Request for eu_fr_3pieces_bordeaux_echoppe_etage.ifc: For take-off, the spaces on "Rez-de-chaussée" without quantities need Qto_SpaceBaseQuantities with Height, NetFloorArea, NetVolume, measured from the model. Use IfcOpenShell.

First a look at what the model holds.

```python
import ifcopenshell
import ifcopenshell.util.element
import ifcopenshell.util.unit

model = ifcopenshell.open("eu_fr_3pieces_bordeaux_echoppe_etage.ifc")
print(model.schema)
for unit_type in ("LENGTHUNIT", "AREAUNIT", "VOLUMEUNIT"):
    print(unit_type, ifcopenshell.util.unit.calculate_unit_scale(model, unit_type))
storey = next(s for s in model.by_type("IfcBuildingStorey") if s.Name == "Rez-de-chaussée")
spaces = [e for e in ifcopenshell.util.element.get_decomposition(storey) if e.is_a("IfcSpace")]
for e in sorted(spaces, key=lambda e: e.id()):
    print(e.id(), e.is_a(), e.Name, list(ifcopenshell.util.element.get_psets(e, qtos_only=True)), sep=" | ")
```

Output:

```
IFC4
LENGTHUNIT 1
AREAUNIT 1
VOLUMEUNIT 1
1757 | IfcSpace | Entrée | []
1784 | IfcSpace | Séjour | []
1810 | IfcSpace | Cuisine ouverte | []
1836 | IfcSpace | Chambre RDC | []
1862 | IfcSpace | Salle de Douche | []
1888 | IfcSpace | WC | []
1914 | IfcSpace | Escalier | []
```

```python
import ifcopenshell
import ifcopenshell.api.pset
import ifcopenshell.geom
import ifcopenshell.util.element
import ifcopenshell.util.shape
import ifcopenshell.util.unit

model = ifcopenshell.open("eu_fr_3pieces_bordeaux_echoppe_etage.ifc")
unit_scale = ifcopenshell.util.unit.calculate_unit_scale(model)
area_scale = ifcopenshell.util.unit.calculate_unit_scale(model, "AREAUNIT")
volume_scale = ifcopenshell.util.unit.calculate_unit_scale(model, "VOLUMEUNIT")
settings = ifcopenshell.geom.settings()

storey = next(s for s in model.by_type("IfcBuildingStorey") if s.Name == "Rez-de-chaussée")
spaces = [e for e in ifcopenshell.util.element.get_decomposition(storey) if e.is_a("IfcSpace")]

for e in sorted(spaces, key=lambda e: e.id()):
    if ifcopenshell.util.element.get_psets(e, qtos_only=True, should_inherit=False):
        continue
    # Geometry comes back in metres, in the element's own axes.
    shape = ifcopenshell.geom.create_shape(settings, e)
    values = {
        "Height": ifcopenshell.util.shape.get_z(shape.geometry) / unit_scale,
        "NetFloorArea": ifcopenshell.util.shape.get_footprint_area(shape.geometry) / area_scale,
        "NetVolume": ifcopenshell.util.shape.get_volume(shape.geometry) / volume_scale,
    }
    qto = ifcopenshell.api.pset.add_qto(model, product=e, name="Qto_SpaceBaseQuantities")
    ifcopenshell.api.pset.edit_qto(model, qto=qto, properties=values)
    print(e.id(), {k: round(v, 3) for k, v in values.items()})

model.write("eu_fr_3pieces_bordeaux_echoppe_etage_v2.ifc")
```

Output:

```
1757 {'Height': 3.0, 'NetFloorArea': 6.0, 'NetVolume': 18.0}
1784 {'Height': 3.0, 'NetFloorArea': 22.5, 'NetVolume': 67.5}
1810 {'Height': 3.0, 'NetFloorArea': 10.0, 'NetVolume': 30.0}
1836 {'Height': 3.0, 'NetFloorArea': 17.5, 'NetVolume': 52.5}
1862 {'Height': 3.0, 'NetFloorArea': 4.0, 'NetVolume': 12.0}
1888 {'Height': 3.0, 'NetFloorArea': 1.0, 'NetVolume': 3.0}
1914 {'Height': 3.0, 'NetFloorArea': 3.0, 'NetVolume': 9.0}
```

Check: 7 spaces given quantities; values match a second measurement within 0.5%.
